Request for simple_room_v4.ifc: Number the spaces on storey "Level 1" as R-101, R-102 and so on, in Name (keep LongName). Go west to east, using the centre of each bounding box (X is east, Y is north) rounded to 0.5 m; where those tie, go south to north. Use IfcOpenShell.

First a look at what the model holds.

```python
import ifcopenshell
import ifcopenshell.util.element
import ifcopenshell.util.placement

model = ifcopenshell.open("simple_room_v4.ifc")
print(model.schema)
storey = next(s for s in model.by_type("IfcBuildingStorey") if s.Name == "Level 1")
spaces = [e for e in ifcopenshell.util.element.get_decomposition(storey) if e.is_a("IfcSpace")]
for e in sorted(spaces, key=lambda e: e.id()):
    origin = ifcopenshell.util.placement.get_local_placement(e.ObjectPlacement)[:3, 3]
    print(e.id(), e.Name, e.LongName, origin.round(2) + 0.0, sep=" | ")
```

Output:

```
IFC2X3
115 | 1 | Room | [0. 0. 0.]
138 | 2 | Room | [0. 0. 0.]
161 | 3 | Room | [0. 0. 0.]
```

```python
import ifcopenshell
import ifcopenshell.geom
import ifcopenshell.util.element
import ifcopenshell.util.shape

model = ifcopenshell.open("simple_room_v4.ifc")
settings = ifcopenshell.geom.settings()
settings.set("use-world-coords", True)


def centre(element):
    shape = ifcopenshell.geom.create_shape(settings, element)
    return ifcopenshell.util.shape.get_bbox_centroid(shape.geometry)


storey = next(s for s in model.by_type("IfcBuildingStorey") if s.Name == "Level 1")
spaces = [e for e in ifcopenshell.util.element.get_decomposition(storey) if e.is_a("IfcSpace")]

# Insertion points can sit at a corner or the storey origin, so sort by the geometry (in metres).
centres = {e: centre(e) for e in spaces}
spaces.sort(key=lambda e: (round(centres[e][0] / 0.5), centres[e][1]))

for i, e in enumerate(spaces, start=1):
    number = f"R-1{i:02d}"
    e.Name = number
    print(e.id(), number)

model.write("simple_room_v4_v2.ifc")
```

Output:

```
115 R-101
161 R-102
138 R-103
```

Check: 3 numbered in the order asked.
